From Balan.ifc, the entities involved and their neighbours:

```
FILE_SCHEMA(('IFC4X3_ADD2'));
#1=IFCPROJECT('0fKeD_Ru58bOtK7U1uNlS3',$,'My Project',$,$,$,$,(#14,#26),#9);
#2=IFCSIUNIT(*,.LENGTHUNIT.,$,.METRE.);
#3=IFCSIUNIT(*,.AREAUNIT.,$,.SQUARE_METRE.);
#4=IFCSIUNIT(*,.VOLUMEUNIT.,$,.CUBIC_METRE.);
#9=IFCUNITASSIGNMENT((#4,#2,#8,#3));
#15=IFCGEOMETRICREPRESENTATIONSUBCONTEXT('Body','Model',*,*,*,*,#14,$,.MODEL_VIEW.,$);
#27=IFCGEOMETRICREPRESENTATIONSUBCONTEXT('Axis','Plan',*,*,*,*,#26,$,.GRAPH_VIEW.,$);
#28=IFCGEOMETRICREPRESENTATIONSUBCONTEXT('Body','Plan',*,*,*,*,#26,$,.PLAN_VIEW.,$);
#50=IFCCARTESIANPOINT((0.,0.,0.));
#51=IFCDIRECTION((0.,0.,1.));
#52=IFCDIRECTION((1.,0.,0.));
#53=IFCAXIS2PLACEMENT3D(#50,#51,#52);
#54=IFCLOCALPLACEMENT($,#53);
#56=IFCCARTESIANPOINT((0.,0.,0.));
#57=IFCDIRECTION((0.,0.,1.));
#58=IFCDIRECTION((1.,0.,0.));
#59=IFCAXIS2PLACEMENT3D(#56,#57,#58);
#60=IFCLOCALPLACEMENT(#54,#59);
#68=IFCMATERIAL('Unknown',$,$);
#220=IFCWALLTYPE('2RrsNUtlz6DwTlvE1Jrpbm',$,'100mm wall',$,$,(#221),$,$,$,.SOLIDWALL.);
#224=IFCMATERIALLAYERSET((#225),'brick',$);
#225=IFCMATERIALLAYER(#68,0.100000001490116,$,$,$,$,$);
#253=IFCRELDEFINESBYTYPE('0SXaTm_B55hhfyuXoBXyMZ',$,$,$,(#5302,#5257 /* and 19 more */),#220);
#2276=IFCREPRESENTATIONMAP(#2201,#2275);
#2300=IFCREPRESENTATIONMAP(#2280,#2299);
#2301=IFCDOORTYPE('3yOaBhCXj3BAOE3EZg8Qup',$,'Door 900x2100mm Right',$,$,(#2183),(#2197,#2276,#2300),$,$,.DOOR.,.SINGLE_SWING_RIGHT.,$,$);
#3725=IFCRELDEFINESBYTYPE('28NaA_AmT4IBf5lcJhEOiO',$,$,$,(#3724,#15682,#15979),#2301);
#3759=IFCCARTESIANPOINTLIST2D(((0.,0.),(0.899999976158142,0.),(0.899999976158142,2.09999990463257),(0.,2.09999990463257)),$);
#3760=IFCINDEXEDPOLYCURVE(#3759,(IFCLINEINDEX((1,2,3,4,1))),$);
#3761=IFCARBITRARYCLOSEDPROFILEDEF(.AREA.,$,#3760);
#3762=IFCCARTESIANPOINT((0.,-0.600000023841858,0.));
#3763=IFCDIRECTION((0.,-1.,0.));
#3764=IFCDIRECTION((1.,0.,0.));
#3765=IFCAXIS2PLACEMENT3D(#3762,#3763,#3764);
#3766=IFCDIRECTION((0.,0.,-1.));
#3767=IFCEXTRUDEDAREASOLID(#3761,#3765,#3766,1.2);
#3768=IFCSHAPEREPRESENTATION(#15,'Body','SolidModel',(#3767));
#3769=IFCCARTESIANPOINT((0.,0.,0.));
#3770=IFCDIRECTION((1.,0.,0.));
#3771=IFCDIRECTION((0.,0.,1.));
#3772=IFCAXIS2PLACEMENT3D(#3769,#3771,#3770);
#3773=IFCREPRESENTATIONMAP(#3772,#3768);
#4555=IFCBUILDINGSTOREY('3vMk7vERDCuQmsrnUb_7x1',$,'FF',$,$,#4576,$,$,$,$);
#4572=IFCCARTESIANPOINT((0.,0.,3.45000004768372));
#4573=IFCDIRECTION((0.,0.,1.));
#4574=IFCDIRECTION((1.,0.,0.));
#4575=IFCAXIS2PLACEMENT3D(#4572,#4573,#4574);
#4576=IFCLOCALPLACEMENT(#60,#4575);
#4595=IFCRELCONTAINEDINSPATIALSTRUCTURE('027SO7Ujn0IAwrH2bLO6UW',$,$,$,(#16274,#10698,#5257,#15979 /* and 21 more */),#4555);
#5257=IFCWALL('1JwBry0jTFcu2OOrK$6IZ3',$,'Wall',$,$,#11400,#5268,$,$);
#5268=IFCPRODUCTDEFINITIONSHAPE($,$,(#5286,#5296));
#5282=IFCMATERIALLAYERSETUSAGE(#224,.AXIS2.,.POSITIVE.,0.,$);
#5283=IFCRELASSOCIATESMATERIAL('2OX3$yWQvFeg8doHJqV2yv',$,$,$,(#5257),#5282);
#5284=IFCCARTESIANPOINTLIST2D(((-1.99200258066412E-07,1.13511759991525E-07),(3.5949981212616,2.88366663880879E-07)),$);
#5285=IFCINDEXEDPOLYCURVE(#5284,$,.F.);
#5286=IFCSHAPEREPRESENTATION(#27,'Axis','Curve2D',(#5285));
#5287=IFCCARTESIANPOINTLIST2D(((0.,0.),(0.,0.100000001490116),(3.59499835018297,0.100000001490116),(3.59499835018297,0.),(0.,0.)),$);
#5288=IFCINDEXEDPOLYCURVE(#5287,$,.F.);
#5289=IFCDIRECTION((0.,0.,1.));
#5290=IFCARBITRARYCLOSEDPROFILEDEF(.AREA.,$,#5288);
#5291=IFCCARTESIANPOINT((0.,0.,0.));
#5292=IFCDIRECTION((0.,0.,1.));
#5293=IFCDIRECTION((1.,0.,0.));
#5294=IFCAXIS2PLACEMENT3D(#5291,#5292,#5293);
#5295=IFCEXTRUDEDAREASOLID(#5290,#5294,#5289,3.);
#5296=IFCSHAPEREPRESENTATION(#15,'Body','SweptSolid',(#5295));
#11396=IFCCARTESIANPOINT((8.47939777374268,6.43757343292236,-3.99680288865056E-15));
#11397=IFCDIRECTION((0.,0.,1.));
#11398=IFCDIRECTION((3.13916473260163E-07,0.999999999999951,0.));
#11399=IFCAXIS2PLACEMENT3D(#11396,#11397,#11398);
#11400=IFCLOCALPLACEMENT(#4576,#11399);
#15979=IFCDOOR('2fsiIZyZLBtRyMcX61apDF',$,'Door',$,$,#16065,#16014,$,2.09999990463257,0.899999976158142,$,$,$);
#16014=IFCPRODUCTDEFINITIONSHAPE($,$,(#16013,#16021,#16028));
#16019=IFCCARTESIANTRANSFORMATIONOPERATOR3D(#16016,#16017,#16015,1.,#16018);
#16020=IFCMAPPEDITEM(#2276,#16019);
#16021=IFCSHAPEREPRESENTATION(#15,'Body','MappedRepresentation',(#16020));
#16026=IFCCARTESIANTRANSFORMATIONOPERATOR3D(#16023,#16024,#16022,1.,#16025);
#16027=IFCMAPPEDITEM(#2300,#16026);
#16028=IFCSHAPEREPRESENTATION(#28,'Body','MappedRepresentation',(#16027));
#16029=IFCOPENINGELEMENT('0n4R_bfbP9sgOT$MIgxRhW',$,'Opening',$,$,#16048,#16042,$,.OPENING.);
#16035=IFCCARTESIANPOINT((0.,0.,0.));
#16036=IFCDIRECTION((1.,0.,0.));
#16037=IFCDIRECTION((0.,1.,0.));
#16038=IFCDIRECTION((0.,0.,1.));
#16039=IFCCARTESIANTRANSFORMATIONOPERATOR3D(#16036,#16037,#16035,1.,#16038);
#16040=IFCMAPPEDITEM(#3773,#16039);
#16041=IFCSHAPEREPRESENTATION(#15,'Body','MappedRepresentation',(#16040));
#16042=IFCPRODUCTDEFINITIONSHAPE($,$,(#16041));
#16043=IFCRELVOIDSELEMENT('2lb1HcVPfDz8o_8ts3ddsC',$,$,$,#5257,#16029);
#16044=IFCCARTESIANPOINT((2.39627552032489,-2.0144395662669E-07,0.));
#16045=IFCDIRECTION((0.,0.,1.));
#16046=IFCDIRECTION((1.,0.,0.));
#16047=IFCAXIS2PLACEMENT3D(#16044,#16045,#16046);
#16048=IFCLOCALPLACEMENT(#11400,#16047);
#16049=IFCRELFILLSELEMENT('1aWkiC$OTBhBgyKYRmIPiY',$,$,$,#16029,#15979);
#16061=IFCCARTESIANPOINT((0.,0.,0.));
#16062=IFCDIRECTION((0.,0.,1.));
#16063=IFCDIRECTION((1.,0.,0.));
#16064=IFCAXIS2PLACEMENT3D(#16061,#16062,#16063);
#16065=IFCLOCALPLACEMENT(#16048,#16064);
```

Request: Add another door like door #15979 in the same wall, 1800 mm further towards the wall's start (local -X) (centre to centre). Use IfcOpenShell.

```python
import ifcopenshell
import ifcopenshell.api.feature
import ifcopenshell.api.geometry
import ifcopenshell.api.root
import ifcopenshell.geom
import ifcopenshell.util.element
import ifcopenshell.util.placement
import ifcopenshell.util.shape
import ifcopenshell.util.unit

model = ifcopenshell.open("Balan.ifc")
unit_scale = ifcopenshell.util.unit.calculate_unit_scale(model)
settings = ifcopenshell.geom.settings()


def volume(element):
    """Net volume in cubic metres, openings subtracted."""
    shape = ifcopenshell.geom.create_shape(settings, element)
    return ifcopenshell.util.shape.get_volume(shape.geometry)


door = model.by_id(15979)
opening = door.FillsVoids[0].RelatingOpeningElement
wall = opening.VoidsElements[0].RelatingBuildingElement
before = volume(wall)
shift = ifcopenshell.util.placement.get_local_placement(wall.ObjectPlacement)[:3, 0] * -1.8 / unit_scale

# copy_class copies the void relationship, type, container and properties, but no geometry.
new_opening = ifcopenshell.api.root.copy_class(model, product=opening)
new_opening.Representation = ifcopenshell.util.element.copy_deep(
    model, opening.Representation, exclude=["IfcGeometricRepresentationContext", "IfcRepresentationMap"]
)
new_door = ifcopenshell.api.root.copy_class(model, product=door)
new_door.Representation = ifcopenshell.util.element.copy_deep(
    model, door.Representation, exclude=["IfcGeometricRepresentationContext", "IfcRepresentationMap"]
)
ifcopenshell.api.feature.add_filling(model, opening=new_opening, element=new_door)

for old, new in ((opening, new_opening), (door, new_door)):
    matrix = ifcopenshell.util.placement.get_local_placement(old.ObjectPlacement)
    matrix[:3, 3] += shift
    ifcopenshell.api.geometry.edit_object_placement(model, product=new, matrix=matrix, is_si=False)

after = volume(wall)

print(f"wall volume {before:.3f} -> {after:.3f} m3")

model.write("Balan_updated.ifc")
```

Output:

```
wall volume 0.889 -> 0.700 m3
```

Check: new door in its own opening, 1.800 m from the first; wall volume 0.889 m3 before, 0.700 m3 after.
